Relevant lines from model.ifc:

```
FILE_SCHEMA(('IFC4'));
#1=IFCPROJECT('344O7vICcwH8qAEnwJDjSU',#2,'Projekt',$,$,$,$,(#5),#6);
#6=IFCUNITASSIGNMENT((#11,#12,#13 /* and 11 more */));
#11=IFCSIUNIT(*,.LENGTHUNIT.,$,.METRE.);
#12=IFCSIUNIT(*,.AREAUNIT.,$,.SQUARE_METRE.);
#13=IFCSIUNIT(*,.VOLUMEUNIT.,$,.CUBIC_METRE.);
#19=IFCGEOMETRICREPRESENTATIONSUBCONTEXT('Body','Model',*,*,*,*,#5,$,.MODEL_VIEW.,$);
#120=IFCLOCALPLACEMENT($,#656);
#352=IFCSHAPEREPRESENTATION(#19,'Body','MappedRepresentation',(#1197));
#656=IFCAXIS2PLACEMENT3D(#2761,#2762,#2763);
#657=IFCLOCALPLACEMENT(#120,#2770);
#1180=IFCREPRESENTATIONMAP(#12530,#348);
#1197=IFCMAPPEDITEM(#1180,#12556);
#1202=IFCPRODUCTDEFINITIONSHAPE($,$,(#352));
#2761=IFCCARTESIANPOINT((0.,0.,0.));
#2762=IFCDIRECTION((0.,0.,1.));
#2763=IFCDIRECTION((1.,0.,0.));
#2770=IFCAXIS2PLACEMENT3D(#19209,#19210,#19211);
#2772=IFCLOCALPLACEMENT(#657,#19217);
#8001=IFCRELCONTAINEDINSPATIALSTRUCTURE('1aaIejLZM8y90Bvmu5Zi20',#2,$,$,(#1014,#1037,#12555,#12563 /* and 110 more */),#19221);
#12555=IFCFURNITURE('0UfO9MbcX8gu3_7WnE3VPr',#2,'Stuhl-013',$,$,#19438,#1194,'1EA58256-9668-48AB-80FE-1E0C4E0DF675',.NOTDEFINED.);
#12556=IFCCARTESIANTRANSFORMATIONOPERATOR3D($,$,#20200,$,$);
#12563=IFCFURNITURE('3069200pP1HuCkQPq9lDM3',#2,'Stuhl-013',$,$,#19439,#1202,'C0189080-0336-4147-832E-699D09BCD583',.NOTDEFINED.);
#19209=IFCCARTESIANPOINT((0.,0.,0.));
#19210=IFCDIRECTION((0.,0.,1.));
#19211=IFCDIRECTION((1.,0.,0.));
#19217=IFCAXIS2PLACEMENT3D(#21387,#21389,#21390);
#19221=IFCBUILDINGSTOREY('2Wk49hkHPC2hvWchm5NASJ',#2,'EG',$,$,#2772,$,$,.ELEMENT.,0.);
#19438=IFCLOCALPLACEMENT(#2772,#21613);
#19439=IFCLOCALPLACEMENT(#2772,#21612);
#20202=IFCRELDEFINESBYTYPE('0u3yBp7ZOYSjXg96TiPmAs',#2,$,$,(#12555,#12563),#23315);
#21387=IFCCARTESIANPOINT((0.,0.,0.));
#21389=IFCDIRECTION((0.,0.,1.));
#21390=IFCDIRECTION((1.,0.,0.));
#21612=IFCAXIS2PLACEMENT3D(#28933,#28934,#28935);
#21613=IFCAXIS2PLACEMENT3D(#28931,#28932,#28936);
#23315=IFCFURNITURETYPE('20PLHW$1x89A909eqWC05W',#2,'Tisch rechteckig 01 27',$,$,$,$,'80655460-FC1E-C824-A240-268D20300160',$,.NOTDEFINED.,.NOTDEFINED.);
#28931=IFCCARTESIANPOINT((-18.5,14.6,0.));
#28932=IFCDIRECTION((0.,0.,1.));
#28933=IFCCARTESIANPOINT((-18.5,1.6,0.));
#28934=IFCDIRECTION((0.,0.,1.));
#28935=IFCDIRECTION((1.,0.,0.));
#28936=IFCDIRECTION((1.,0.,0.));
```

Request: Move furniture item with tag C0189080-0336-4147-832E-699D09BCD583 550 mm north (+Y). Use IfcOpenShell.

```python
import ifcopenshell
import ifcopenshell.api.geometry
import ifcopenshell.util.placement
import ifcopenshell.util.unit

model = ifcopenshell.open("model.ifc")
unit_scale = ifcopenshell.util.unit.calculate_unit_scale(model)

item = model.by_guid("3069200pP1HuCkQPq9lDM3")
matrix = ifcopenshell.util.placement.get_local_placement(item.ObjectPlacement)
matrix[1, 3] += 0.55 / unit_scale
ifcopenshell.api.geometry.edit_object_placement(model, product=item, matrix=matrix, is_si=False)

print(ifcopenshell.util.placement.get_local_placement(item.ObjectPlacement).round(3) + 0.0)

model.write("model_v2.ifc")
```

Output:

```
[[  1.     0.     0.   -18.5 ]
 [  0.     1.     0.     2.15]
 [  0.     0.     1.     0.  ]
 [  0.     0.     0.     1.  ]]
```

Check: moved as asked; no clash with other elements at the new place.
